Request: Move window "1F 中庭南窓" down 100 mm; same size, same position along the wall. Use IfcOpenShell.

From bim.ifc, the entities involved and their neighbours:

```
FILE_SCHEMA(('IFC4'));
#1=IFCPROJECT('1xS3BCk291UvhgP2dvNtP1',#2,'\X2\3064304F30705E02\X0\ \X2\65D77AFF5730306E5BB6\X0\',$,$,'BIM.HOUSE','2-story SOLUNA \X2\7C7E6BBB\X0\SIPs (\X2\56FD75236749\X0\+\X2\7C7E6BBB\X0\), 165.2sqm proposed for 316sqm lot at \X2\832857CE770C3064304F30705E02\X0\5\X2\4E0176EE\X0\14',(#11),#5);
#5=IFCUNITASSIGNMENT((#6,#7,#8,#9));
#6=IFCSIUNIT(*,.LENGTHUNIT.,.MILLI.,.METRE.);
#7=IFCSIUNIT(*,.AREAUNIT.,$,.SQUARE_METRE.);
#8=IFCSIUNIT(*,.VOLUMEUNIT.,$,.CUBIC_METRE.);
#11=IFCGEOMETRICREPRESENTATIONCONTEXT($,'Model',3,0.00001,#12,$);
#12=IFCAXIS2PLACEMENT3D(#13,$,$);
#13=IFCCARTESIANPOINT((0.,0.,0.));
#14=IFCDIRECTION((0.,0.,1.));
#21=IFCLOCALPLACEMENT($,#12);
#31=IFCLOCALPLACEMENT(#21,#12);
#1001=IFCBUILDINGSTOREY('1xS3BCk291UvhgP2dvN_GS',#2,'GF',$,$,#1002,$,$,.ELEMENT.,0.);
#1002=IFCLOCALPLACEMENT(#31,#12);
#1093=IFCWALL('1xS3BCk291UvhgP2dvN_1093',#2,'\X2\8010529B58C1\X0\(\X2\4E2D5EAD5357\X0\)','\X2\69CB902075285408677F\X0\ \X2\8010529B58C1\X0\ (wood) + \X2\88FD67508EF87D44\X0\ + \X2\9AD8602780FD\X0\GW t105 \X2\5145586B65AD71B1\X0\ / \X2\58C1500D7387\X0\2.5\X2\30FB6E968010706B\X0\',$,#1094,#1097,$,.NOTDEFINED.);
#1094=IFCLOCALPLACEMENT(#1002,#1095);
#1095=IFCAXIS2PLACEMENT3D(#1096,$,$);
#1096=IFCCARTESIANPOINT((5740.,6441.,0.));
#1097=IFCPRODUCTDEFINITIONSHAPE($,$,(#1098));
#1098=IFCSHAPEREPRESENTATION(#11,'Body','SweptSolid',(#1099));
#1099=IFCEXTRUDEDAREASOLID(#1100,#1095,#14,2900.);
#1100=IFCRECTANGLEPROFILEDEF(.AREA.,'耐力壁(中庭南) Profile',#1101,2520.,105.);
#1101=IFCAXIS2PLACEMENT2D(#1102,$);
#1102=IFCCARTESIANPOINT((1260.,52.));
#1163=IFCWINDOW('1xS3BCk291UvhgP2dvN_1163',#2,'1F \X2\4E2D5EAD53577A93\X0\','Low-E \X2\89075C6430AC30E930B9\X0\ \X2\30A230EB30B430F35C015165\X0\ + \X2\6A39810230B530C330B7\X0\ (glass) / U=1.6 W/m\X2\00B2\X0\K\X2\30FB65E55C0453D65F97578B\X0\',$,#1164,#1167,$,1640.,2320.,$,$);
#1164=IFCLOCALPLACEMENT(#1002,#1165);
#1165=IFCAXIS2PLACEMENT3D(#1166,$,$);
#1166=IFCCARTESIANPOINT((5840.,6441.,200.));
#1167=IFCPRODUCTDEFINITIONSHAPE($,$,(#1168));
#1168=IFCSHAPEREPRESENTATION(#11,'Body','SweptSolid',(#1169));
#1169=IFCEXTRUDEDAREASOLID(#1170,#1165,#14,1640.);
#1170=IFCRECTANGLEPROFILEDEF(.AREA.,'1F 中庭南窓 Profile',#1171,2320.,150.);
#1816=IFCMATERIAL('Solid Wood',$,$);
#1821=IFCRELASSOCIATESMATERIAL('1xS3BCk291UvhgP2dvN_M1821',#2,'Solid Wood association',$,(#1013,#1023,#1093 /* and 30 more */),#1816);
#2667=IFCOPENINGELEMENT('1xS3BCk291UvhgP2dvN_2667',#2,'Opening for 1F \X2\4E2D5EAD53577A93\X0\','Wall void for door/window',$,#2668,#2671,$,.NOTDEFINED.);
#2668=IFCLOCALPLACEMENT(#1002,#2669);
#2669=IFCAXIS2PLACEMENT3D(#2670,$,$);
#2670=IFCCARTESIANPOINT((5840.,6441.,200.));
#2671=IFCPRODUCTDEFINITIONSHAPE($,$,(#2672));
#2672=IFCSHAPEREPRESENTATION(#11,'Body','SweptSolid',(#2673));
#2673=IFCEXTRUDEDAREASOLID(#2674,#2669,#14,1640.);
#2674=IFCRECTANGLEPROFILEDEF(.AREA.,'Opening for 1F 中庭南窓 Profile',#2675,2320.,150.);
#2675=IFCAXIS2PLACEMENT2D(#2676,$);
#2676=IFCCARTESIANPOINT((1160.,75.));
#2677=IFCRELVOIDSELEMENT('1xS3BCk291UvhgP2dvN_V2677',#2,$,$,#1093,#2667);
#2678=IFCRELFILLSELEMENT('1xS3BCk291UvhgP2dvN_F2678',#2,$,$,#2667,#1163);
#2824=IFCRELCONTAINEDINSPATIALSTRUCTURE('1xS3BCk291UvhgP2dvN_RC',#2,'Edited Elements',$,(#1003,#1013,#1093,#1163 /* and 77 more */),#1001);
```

```python
import numpy as np
import ifcopenshell
import ifcopenshell.api.geometry
import ifcopenshell.util.placement
import ifcopenshell.util.unit

model = ifcopenshell.open("bim.ifc")
unit_scale = ifcopenshell.util.unit.calculate_unit_scale(model)

window = model.by_guid("1xS3BCk291UvhgP2dvN_1163")
opening = window.FillsVoids[0].RelatingOpeningElement
dz = -0.1 / unit_scale

shift = np.array([0.0, 0.0, dz])
# The window is not placed relative to its opening, so move both.
for product in (opening, window):
    matrix = ifcopenshell.util.placement.get_local_placement(product.ObjectPlacement)
    matrix[:3, 3] += shift
    ifcopenshell.api.geometry.edit_object_placement(model, product=product, matrix=matrix, is_si=False)

print(f"moved by {dz * unit_scale:+.3f} m")

model.write("bim_updated.ifc")
```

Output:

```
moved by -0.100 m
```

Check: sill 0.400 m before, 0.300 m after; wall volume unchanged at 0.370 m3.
